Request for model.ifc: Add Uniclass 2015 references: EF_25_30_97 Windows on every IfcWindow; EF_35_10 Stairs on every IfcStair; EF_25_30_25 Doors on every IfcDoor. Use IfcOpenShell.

First a look at what the model holds.

```python
import ifcopenshell

model = ifcopenshell.open("model.ifc")
print(model.schema)
print("classifications:", [c.Name for c in model.by_type("IfcClassification")])
for ifc_class in ("IfcDoor", "IfcRoof", "IfcStair", "IfcWall", "IfcWindow"):
    print(ifc_class, len(model.by_type(ifc_class)))
```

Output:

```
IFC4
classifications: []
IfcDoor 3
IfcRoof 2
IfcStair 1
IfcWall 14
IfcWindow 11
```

```python
import ifcopenshell
import ifcopenshell.api.classification

model = ifcopenshell.open("model.ifc")

system = ifcopenshell.api.classification.add_classification(model, classification="Uniclass 2015")

codes = {
    "IfcWindow": ("EF_25_30_97", "Windows"),
    "IfcStair": ("EF_35_10", "Stairs"),
    "IfcDoor": ("EF_25_30_25", "Doors"),
}
for ifc_class, (code, name) in codes.items():
    products = model.by_type(ifc_class)
    ifcopenshell.api.classification.add_reference(
        model, products=products, classification=system, identification=code, name=name
    )
    print(code, len(products))

model.write("model-out.ifc")
```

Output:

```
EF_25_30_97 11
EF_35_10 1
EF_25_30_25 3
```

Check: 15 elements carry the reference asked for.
